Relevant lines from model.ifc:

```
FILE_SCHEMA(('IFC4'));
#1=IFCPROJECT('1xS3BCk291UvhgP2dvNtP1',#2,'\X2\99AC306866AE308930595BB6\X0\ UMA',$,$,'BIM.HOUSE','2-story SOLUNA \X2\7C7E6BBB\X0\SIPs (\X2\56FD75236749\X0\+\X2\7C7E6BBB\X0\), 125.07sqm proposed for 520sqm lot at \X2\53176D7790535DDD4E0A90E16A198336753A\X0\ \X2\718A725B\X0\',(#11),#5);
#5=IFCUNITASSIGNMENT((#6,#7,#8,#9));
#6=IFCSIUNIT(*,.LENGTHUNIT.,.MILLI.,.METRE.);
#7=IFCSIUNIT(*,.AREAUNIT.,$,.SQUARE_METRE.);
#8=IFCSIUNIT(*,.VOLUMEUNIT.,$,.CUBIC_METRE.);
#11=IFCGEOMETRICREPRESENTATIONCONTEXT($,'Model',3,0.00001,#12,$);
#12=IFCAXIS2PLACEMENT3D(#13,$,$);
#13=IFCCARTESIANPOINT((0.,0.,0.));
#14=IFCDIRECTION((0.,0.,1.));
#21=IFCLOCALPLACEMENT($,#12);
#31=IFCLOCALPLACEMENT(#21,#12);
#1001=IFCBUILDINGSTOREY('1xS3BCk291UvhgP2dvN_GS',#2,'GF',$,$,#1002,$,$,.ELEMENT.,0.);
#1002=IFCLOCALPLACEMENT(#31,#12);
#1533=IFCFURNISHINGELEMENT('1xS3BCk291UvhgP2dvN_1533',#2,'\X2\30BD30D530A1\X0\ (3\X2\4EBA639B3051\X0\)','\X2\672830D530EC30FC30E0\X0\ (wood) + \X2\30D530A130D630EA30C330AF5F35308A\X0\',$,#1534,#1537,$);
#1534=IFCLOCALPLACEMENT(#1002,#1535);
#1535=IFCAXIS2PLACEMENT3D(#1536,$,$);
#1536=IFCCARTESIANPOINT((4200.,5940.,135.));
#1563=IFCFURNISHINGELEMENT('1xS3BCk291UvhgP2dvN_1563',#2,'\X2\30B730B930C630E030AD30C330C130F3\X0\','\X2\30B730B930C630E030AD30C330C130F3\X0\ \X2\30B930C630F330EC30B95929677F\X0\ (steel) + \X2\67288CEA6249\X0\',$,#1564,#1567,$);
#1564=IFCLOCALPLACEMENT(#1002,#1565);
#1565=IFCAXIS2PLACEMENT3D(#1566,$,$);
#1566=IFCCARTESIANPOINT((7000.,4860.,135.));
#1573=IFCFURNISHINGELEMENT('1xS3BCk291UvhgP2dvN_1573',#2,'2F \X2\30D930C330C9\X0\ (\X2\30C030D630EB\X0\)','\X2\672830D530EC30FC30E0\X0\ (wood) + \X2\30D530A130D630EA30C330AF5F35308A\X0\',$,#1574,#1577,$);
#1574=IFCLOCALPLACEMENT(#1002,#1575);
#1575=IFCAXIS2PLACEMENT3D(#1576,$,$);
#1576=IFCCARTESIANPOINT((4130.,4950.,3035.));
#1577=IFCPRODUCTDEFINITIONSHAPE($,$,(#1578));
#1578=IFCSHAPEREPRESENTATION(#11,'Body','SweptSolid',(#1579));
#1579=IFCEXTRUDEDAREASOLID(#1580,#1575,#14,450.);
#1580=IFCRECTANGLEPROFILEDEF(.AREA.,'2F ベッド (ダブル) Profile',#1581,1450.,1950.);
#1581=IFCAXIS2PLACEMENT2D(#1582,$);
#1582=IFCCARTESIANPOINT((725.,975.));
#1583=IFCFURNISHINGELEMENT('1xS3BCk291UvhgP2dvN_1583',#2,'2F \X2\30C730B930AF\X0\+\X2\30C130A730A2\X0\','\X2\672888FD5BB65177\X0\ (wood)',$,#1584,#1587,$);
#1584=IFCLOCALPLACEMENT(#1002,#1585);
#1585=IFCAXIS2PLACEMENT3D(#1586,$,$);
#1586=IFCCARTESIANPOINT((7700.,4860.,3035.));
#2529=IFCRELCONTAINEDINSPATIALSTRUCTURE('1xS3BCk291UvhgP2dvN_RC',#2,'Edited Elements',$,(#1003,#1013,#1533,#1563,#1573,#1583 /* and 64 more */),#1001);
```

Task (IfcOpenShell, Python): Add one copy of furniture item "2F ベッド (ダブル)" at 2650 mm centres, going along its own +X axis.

```python
import ifcopenshell
import ifcopenshell.api.geometry
import ifcopenshell.api.root
import ifcopenshell.util.element
import ifcopenshell.util.placement
import ifcopenshell.util.unit

model = ifcopenshell.open("model.ifc")
unit_scale = ifcopenshell.util.unit.calculate_unit_scale(model)


def reuse_history(source, copy):
    """copy_class also copies each property set's owner history, people and application; keep the originals."""
    for rel in copy.IsDefinedBy:
        if rel.is_a("IfcRelDefinesByProperties") and (history := rel.RelatingPropertyDefinition.OwnerHistory):
            rel.RelatingPropertyDefinition.OwnerHistory = source.OwnerHistory
            ifcopenshell.util.element.remove_deep2(model, history)


source = model.by_guid("1xS3BCk291UvhgP2dvN_1573")
base = ifcopenshell.util.placement.get_local_placement(source.ObjectPlacement)
step = base[:3, 0] * 2.65 / unit_scale

for i in range(1, 2):
    copy = ifcopenshell.api.root.copy_class(model, product=source)
    copy.Representation = ifcopenshell.util.element.copy_deep(
        model, source.Representation, exclude=["IfcGeometricRepresentationContext", "IfcRepresentationMap"]
    )
    reuse_history(source, copy)
    matrix = base.copy()
    matrix[:3, 3] += i * step
    print("added at", matrix[:3, 3].round(3) + 0.0)
    ifcopenshell.api.geometry.edit_object_placement(model, product=copy, matrix=matrix, is_si=False)

model.write("model-out.ifc")
```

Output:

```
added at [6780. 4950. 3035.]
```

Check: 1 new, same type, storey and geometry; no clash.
